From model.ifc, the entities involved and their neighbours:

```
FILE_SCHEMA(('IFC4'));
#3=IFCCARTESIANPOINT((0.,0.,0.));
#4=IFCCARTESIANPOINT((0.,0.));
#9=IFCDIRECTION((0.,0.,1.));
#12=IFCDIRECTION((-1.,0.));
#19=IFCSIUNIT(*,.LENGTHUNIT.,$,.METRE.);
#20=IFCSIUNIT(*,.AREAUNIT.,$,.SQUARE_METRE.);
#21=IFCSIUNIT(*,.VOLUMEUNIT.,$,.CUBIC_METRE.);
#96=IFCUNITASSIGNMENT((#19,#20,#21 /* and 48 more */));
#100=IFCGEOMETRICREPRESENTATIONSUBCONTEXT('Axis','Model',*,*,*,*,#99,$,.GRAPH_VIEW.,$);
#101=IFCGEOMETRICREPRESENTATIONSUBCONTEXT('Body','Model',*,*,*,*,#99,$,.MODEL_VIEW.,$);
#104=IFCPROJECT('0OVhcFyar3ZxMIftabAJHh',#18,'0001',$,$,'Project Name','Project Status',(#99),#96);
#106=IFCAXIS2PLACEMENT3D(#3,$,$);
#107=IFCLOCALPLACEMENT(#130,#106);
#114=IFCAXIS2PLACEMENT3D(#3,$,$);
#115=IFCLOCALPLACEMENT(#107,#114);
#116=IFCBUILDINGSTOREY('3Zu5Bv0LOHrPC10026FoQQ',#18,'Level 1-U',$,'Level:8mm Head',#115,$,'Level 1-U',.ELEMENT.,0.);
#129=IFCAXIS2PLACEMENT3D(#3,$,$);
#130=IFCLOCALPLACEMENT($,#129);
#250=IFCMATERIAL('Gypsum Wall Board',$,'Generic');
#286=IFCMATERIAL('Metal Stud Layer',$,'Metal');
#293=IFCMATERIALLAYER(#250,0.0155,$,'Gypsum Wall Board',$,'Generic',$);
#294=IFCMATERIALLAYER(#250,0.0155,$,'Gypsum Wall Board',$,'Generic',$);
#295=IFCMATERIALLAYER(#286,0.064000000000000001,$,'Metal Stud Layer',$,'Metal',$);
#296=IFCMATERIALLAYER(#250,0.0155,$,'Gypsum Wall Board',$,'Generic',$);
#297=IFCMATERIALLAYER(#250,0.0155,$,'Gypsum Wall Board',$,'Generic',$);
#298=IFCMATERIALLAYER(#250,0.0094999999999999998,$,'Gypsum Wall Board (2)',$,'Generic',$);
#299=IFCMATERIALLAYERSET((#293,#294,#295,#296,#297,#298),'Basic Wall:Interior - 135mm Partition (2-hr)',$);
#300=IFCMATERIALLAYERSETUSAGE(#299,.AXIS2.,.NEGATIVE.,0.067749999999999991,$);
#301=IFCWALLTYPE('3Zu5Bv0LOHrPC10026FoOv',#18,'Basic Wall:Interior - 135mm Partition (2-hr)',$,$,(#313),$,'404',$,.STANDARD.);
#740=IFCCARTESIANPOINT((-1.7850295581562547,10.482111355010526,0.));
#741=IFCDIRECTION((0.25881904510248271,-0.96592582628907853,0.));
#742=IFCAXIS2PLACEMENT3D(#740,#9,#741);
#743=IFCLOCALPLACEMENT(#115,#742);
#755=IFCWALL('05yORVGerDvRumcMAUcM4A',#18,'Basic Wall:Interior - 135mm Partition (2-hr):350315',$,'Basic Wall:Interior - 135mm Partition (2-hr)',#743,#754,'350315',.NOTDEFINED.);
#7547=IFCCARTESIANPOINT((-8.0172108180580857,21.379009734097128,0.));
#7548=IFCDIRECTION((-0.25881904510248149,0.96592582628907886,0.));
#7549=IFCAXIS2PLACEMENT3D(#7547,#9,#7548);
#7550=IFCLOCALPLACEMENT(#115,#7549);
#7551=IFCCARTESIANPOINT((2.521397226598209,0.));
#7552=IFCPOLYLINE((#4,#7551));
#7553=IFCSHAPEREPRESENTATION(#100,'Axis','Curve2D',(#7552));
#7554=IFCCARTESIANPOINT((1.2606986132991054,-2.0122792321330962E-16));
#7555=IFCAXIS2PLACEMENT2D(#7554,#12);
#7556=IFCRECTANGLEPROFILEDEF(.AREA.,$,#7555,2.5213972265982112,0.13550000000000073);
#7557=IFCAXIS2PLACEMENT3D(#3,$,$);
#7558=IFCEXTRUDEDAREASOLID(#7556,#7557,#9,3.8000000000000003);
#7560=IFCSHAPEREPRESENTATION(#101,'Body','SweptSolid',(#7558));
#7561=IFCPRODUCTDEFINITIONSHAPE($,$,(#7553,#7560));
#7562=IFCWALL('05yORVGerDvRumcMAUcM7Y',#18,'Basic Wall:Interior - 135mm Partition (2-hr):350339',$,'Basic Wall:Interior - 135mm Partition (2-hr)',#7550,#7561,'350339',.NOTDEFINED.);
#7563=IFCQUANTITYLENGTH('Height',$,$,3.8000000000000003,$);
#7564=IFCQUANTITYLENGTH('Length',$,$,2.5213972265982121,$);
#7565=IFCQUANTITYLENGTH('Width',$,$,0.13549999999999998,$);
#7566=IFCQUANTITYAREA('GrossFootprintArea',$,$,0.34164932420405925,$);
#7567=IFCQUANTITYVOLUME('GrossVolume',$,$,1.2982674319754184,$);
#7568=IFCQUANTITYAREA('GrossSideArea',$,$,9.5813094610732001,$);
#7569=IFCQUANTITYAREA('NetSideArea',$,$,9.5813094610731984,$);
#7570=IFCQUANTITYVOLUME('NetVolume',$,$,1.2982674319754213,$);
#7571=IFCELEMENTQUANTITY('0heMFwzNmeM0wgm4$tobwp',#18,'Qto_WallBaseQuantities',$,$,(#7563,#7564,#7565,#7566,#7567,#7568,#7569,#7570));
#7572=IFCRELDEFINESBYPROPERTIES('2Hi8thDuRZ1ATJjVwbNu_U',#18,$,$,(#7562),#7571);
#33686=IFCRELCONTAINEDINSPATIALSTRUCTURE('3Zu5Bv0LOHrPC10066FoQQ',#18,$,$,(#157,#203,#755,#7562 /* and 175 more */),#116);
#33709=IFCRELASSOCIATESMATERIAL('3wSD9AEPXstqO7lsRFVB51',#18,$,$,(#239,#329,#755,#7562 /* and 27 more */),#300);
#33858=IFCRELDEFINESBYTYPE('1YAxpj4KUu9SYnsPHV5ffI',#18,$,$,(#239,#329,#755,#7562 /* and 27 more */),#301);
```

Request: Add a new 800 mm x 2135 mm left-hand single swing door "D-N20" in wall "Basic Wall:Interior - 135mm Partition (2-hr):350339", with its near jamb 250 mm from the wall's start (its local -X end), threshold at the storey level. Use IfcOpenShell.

```python
import numpy as np
import ifcopenshell
import ifcopenshell.api.feature
import ifcopenshell.api.geometry
import ifcopenshell.api.pset
import ifcopenshell.api.root
import ifcopenshell.api.spatial
import ifcopenshell.geom
import ifcopenshell.util.element
import ifcopenshell.util.placement
import ifcopenshell.util.representation
import ifcopenshell.util.shape
import ifcopenshell.util.unit

model = ifcopenshell.open("model.ifc")
unit_scale = ifcopenshell.util.unit.calculate_unit_scale(model)
area_scale = ifcopenshell.util.unit.calculate_unit_scale(model, "AREAUNIT")
volume_scale = ifcopenshell.util.unit.calculate_unit_scale(model, "VOLUMEUNIT")
settings = ifcopenshell.geom.settings()


def volume(element):
    """Net volume in cubic metres, openings subtracted."""
    shape = ifcopenshell.geom.create_shape(settings, element)
    return ifcopenshell.util.shape.get_volume(shape.geometry)


wall = model.by_id(7562)
storey = ifcopenshell.util.element.get_container(wall, ifc_class="IfcBuildingStorey")
context = ifcopenshell.util.representation.get_context(model, "Model", "Body", "MODEL_VIEW")
before = volume(wall)

width, height, from_end, sill = 0.8, 2.135, 0.25, 0.0  # metres

# The wall runs along its own X axis, and the end named is its -X end.
wall_shape = ifcopenshell.geom.create_shape(settings, wall)
x, y, z = ifcopenshell.util.shape.get_vertices(wall_shape.geometry).T
start = x.min() + from_end
face, thickness = float(y.min()), float(y.max() - y.min())
wall_matrix = ifcopenshell.util.placement.get_local_placement(wall.ObjectPlacement)
level = ifcopenshell.util.placement.get_local_placement(storey.ObjectPlacement)[2, 3]


def in_wall(x, y):
    """Placement at x, y metres in the wall's axes, at sill height."""
    matrix = wall_matrix.copy()
    matrix[:, 3] = wall_matrix @ np.array([x / unit_scale, y / unit_scale, 0.0, 1.0])
    matrix[2, 3] = level + sill / unit_scale
    return matrix


# Opening: a box that overshoots both wall faces by 50 mm.
opening = ifcopenshell.api.root.create_entity(model, ifc_class="IfcOpeningElement", predefined_type="OPENING")
box = ifcopenshell.api.geometry.add_wall_representation(
    model, context=context, length=width, height=height, thickness=thickness + 0.1
)
ifcopenshell.api.geometry.assign_representation(model, product=opening, representation=box)
ifcopenshell.api.geometry.edit_object_placement(model, product=opening, matrix=in_wall(start, face - 0.05), is_si=False)
ifcopenshell.api.feature.add_feature(model, feature=opening, element=wall)

door = ifcopenshell.api.root.create_entity(model, ifc_class="IfcDoor", name="D-N20", predefined_type="DOOR")
door.OverallWidth, door.OverallHeight = width / unit_scale, height / unit_scale
door.OperationType = "SINGLE_SWING_LEFT"
body = ifcopenshell.api.geometry.add_door_representation(
    model,
    context=context,
    overall_width=door.OverallWidth,
    overall_height=door.OverallHeight,
    operation_type="SINGLE_SWING_LEFT",
    lining_properties={"LiningDepth": thickness / unit_scale, "ThresholdDepth": thickness / unit_scale},
)
ifcopenshell.api.geometry.assign_representation(model, product=door, representation=body)
ifcopenshell.api.spatial.assign_container(model, products=[door], relating_structure=storey)
ifcopenshell.api.feature.add_filling(model, opening=opening, element=door)

# The lining spans the wall, so the door starts at the wall face.
ifcopenshell.api.geometry.edit_object_placement(model, product=door, matrix=in_wall(start, face), is_si=False)

after = volume(wall)

# Update the wall's stored quantities.
qto = model.by_id(ifcopenshell.util.element.get_pset(wall, "Qto_WallBaseQuantities", should_inherit=False)["id"])
ifcopenshell.api.pset.edit_qto(model, qto=qto, properties={
    "NetSideArea": after / thickness / area_scale,
    "NetVolume": after / volume_scale,
})

print(f"wall volume {before:.3f} -> {after:.3f} m3")

model.write("model_updated.ifc")
```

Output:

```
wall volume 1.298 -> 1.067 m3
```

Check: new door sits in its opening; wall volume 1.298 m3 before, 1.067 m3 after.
